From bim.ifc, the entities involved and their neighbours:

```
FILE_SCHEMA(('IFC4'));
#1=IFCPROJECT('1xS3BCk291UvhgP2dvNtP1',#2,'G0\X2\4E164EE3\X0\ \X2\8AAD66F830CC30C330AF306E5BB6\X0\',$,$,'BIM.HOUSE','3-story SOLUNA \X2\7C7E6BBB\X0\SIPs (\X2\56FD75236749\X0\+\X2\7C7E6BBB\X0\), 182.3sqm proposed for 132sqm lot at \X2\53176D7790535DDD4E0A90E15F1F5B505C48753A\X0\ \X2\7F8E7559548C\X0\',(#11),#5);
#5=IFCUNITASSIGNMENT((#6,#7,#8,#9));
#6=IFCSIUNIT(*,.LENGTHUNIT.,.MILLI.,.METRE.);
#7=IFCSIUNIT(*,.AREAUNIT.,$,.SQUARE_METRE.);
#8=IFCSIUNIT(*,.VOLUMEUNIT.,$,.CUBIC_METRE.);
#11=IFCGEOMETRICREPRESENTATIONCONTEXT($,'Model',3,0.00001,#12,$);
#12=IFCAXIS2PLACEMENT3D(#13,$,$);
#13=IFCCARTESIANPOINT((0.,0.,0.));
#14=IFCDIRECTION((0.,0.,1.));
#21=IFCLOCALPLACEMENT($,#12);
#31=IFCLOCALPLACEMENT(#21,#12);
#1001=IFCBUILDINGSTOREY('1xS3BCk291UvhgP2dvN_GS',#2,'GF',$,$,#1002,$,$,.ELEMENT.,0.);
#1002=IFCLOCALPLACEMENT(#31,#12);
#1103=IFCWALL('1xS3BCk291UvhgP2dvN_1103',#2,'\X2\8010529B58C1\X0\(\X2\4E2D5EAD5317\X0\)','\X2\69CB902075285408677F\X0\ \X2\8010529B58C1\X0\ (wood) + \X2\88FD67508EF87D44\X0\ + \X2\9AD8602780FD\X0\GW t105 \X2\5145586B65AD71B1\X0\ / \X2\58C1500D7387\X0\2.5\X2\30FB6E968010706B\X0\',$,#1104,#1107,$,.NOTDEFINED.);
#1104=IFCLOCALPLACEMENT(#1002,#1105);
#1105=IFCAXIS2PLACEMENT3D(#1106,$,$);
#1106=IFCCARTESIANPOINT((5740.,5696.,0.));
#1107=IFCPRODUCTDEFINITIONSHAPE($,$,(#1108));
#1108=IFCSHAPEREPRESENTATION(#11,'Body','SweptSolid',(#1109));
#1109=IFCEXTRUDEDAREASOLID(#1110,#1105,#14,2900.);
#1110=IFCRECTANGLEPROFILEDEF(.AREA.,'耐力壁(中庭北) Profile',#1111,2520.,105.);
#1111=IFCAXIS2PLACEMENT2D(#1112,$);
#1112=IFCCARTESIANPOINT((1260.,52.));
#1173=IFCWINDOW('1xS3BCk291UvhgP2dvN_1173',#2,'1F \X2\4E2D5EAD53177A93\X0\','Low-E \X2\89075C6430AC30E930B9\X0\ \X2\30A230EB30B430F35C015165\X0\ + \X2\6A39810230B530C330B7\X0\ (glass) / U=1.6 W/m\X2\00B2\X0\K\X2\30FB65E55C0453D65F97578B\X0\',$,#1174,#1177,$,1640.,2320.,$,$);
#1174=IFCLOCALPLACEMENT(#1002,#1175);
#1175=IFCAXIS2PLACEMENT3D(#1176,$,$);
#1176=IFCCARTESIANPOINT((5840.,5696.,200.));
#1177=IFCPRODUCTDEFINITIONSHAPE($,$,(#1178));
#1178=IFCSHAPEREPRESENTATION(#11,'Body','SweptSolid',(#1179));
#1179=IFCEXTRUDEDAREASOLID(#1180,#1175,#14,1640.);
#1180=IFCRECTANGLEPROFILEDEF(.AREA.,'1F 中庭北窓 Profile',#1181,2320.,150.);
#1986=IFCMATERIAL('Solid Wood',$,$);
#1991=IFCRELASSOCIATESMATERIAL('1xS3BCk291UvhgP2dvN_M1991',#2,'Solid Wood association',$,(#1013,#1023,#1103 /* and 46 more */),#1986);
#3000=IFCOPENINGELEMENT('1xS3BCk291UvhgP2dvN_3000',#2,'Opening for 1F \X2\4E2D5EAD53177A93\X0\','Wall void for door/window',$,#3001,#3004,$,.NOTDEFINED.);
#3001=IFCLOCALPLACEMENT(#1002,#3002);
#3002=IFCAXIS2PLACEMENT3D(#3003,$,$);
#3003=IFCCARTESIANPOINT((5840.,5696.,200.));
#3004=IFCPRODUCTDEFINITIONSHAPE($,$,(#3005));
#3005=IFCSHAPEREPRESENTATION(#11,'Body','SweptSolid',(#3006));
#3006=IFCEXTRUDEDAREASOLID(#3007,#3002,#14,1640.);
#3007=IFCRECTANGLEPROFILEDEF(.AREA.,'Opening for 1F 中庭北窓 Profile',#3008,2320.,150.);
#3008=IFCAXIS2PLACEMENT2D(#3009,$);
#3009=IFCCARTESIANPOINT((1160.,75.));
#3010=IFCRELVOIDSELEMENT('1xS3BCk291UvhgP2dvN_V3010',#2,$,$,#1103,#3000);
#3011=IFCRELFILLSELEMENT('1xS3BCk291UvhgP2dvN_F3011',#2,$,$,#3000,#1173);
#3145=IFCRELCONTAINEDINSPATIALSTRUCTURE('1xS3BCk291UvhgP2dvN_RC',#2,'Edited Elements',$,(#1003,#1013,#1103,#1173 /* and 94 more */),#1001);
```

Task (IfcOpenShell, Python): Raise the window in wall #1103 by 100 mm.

```python
import numpy as np
import ifcopenshell
import ifcopenshell.api.geometry
import ifcopenshell.util.placement
import ifcopenshell.util.unit

model = ifcopenshell.open("bim.ifc")
unit_scale = ifcopenshell.util.unit.calculate_unit_scale(model)

window = model.by_id(1173)
opening = window.FillsVoids[0].RelatingOpeningElement
dz = 0.1 / unit_scale

shift = np.array([0.0, 0.0, dz])
# The window is not placed relative to its opening, so move both.
for product in (opening, window):
    matrix = ifcopenshell.util.placement.get_local_placement(product.ObjectPlacement)
    matrix[:3, 3] += shift
    ifcopenshell.api.geometry.edit_object_placement(model, product=product, matrix=matrix, is_si=False)

print(f"moved by {dz * unit_scale:+.3f} m")

model.write("bim_updated.ifc")
```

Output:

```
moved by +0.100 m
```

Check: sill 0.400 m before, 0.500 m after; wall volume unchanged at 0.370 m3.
